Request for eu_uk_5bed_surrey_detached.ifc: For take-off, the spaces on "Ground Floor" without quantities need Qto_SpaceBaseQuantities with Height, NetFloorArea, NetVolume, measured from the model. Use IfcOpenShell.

First a look at what the model holds.

```python
import ifcopenshell
import ifcopenshell.util.element
import ifcopenshell.util.unit

model = ifcopenshell.open("eu_uk_5bed_surrey_detached.ifc")
print(model.schema)
for unit_type in ("LENGTHUNIT", "AREAUNIT", "VOLUMEUNIT"):
    print(unit_type, ifcopenshell.util.unit.calculate_unit_scale(model, unit_type))
storey = next(s for s in model.by_type("IfcBuildingStorey") if s.Name == "Ground Floor")
spaces = [e for e in ifcopenshell.util.element.get_decomposition(storey) if e.is_a("IfcSpace")]
for e in sorted(spaces, key=lambda e: e.id()):
    print(e.id(), e.is_a(), e.Name, list(ifcopenshell.util.element.get_psets(e, qtos_only=True)), sep=" | ")
```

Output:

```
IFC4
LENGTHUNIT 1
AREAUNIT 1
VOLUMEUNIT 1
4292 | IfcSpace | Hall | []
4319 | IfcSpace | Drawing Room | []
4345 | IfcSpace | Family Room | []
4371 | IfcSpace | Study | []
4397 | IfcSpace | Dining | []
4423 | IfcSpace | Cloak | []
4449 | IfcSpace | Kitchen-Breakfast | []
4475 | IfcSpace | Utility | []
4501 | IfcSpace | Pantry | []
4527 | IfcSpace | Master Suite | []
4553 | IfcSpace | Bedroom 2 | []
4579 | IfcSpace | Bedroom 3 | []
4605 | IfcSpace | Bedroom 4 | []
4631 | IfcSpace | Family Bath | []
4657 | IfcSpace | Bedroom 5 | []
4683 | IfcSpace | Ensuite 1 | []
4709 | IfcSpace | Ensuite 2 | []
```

```python
import ifcopenshell
import ifcopenshell.api.pset
import ifcopenshell.geom
import ifcopenshell.util.element
import ifcopenshell.util.shape
import ifcopenshell.util.unit

model = ifcopenshell.open("eu_uk_5bed_surrey_detached.ifc")
unit_scale = ifcopenshell.util.unit.calculate_unit_scale(model)
area_scale = ifcopenshell.util.unit.calculate_unit_scale(model, "AREAUNIT")
volume_scale = ifcopenshell.util.unit.calculate_unit_scale(model, "VOLUMEUNIT")
settings = ifcopenshell.geom.settings()

storey = next(s for s in model.by_type("IfcBuildingStorey") if s.Name == "Ground Floor")
spaces = [e for e in ifcopenshell.util.element.get_decomposition(storey) if e.is_a("IfcSpace")]

for e in sorted(spaces, key=lambda e: e.id()):
    if ifcopenshell.util.element.get_psets(e, qtos_only=True, should_inherit=False):
        continue
    # Geometry comes back in metres, in the element's own axes.
    shape = ifcopenshell.geom.create_shape(settings, e)
    values = {
        "Height": ifcopenshell.util.shape.get_z(shape.geometry) / unit_scale,
        "NetFloorArea": ifcopenshell.util.shape.get_footprint_area(shape.geometry) / area_scale,
        "NetVolume": ifcopenshell.util.shape.get_volume(shape.geometry) / volume_scale,
    }
    qto = ifcopenshell.api.pset.add_qto(model, product=e, name="Qto_SpaceBaseQuantities")
    ifcopenshell.api.pset.edit_qto(model, qto=qto, properties=values)
    print(e.id(), {k: round(v, 3) for k, v in values.items()})

model.write("eu_uk_5bed_surrey_detached_edited.ifc")
```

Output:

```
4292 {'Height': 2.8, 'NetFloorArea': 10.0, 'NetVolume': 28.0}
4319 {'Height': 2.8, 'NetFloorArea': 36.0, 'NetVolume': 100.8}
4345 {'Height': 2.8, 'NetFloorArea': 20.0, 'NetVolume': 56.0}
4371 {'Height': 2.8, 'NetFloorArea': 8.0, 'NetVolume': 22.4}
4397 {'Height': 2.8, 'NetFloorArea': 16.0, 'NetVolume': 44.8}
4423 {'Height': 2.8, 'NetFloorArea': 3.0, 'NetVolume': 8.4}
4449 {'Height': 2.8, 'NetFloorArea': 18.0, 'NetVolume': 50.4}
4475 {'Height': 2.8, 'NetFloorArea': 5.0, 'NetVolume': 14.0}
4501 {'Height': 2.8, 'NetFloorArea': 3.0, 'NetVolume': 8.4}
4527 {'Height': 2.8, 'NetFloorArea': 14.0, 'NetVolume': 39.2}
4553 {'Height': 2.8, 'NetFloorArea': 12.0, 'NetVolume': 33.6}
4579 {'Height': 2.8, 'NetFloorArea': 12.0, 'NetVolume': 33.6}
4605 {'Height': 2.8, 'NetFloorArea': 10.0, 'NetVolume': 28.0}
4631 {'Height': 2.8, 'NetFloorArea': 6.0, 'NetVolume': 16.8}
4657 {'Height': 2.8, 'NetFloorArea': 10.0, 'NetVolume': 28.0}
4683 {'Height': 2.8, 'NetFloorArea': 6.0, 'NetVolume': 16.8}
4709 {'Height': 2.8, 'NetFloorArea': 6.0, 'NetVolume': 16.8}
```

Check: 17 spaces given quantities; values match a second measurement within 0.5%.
